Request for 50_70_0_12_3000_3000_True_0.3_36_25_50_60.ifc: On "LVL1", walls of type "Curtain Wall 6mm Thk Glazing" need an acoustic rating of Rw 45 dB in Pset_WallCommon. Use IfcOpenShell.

First a look at what the model holds.

```python
import ifcopenshell
import ifcopenshell.util.element

model = ifcopenshell.open("50_70_0_12_3000_3000_True_0.3_36_25_50_60.ifc")
print(model.schema)
storey = next(s for s in model.by_type("IfcBuildingStorey") if s.Name == "LVL1")
walls = [e for e in ifcopenshell.util.element.get_decomposition(storey) if e.is_a("IfcWall")]
seen = {}
for e in walls:
    element_type = ifcopenshell.util.element.get_type(e)
    key = (element_type.Name if element_type != e and element_type else None, ifcopenshell.util.element.get_pset(e, "Pset_WallCommon", "AcousticRating"))
    seen[key] = seen.get(key, 0) + 1
for (name, value), count in sorted(seen.items(), key=str):
    print(count, "x", name, "|", value)
```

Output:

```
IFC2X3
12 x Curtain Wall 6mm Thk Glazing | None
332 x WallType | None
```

```python
import ifcopenshell
import ifcopenshell.api.pset
import ifcopenshell.util.element

model = ifcopenshell.open("50_70_0_12_3000_3000_True_0.3_36_25_50_60.ifc")

storey = next(s for s in model.by_type("IfcBuildingStorey") if s.Name == "LVL1")
walls = [e for e in ifcopenshell.util.element.get_decomposition(storey) if e.is_a("IfcWall")]

count = 0
for e in walls:
    element_type = ifcopenshell.util.element.get_type(e)
    if element_type in (None, e) or element_type.Name != "Curtain Wall 6mm Thk Glazing":
        continue
    # add_pset returns the element's existing set when there is one.
    pset = ifcopenshell.api.pset.add_pset(model, product=e, name="Pset_WallCommon")
    ifcopenshell.api.pset.edit_pset(model, pset=pset, properties={"AcousticRating": "Rw 45 dB"})
    count += 1

print(count, "walls updated")

model.write("50_70_0_12_3000_3000_True_0.3_36_25_50_60_v2.ifc")
```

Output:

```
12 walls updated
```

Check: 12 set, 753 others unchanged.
